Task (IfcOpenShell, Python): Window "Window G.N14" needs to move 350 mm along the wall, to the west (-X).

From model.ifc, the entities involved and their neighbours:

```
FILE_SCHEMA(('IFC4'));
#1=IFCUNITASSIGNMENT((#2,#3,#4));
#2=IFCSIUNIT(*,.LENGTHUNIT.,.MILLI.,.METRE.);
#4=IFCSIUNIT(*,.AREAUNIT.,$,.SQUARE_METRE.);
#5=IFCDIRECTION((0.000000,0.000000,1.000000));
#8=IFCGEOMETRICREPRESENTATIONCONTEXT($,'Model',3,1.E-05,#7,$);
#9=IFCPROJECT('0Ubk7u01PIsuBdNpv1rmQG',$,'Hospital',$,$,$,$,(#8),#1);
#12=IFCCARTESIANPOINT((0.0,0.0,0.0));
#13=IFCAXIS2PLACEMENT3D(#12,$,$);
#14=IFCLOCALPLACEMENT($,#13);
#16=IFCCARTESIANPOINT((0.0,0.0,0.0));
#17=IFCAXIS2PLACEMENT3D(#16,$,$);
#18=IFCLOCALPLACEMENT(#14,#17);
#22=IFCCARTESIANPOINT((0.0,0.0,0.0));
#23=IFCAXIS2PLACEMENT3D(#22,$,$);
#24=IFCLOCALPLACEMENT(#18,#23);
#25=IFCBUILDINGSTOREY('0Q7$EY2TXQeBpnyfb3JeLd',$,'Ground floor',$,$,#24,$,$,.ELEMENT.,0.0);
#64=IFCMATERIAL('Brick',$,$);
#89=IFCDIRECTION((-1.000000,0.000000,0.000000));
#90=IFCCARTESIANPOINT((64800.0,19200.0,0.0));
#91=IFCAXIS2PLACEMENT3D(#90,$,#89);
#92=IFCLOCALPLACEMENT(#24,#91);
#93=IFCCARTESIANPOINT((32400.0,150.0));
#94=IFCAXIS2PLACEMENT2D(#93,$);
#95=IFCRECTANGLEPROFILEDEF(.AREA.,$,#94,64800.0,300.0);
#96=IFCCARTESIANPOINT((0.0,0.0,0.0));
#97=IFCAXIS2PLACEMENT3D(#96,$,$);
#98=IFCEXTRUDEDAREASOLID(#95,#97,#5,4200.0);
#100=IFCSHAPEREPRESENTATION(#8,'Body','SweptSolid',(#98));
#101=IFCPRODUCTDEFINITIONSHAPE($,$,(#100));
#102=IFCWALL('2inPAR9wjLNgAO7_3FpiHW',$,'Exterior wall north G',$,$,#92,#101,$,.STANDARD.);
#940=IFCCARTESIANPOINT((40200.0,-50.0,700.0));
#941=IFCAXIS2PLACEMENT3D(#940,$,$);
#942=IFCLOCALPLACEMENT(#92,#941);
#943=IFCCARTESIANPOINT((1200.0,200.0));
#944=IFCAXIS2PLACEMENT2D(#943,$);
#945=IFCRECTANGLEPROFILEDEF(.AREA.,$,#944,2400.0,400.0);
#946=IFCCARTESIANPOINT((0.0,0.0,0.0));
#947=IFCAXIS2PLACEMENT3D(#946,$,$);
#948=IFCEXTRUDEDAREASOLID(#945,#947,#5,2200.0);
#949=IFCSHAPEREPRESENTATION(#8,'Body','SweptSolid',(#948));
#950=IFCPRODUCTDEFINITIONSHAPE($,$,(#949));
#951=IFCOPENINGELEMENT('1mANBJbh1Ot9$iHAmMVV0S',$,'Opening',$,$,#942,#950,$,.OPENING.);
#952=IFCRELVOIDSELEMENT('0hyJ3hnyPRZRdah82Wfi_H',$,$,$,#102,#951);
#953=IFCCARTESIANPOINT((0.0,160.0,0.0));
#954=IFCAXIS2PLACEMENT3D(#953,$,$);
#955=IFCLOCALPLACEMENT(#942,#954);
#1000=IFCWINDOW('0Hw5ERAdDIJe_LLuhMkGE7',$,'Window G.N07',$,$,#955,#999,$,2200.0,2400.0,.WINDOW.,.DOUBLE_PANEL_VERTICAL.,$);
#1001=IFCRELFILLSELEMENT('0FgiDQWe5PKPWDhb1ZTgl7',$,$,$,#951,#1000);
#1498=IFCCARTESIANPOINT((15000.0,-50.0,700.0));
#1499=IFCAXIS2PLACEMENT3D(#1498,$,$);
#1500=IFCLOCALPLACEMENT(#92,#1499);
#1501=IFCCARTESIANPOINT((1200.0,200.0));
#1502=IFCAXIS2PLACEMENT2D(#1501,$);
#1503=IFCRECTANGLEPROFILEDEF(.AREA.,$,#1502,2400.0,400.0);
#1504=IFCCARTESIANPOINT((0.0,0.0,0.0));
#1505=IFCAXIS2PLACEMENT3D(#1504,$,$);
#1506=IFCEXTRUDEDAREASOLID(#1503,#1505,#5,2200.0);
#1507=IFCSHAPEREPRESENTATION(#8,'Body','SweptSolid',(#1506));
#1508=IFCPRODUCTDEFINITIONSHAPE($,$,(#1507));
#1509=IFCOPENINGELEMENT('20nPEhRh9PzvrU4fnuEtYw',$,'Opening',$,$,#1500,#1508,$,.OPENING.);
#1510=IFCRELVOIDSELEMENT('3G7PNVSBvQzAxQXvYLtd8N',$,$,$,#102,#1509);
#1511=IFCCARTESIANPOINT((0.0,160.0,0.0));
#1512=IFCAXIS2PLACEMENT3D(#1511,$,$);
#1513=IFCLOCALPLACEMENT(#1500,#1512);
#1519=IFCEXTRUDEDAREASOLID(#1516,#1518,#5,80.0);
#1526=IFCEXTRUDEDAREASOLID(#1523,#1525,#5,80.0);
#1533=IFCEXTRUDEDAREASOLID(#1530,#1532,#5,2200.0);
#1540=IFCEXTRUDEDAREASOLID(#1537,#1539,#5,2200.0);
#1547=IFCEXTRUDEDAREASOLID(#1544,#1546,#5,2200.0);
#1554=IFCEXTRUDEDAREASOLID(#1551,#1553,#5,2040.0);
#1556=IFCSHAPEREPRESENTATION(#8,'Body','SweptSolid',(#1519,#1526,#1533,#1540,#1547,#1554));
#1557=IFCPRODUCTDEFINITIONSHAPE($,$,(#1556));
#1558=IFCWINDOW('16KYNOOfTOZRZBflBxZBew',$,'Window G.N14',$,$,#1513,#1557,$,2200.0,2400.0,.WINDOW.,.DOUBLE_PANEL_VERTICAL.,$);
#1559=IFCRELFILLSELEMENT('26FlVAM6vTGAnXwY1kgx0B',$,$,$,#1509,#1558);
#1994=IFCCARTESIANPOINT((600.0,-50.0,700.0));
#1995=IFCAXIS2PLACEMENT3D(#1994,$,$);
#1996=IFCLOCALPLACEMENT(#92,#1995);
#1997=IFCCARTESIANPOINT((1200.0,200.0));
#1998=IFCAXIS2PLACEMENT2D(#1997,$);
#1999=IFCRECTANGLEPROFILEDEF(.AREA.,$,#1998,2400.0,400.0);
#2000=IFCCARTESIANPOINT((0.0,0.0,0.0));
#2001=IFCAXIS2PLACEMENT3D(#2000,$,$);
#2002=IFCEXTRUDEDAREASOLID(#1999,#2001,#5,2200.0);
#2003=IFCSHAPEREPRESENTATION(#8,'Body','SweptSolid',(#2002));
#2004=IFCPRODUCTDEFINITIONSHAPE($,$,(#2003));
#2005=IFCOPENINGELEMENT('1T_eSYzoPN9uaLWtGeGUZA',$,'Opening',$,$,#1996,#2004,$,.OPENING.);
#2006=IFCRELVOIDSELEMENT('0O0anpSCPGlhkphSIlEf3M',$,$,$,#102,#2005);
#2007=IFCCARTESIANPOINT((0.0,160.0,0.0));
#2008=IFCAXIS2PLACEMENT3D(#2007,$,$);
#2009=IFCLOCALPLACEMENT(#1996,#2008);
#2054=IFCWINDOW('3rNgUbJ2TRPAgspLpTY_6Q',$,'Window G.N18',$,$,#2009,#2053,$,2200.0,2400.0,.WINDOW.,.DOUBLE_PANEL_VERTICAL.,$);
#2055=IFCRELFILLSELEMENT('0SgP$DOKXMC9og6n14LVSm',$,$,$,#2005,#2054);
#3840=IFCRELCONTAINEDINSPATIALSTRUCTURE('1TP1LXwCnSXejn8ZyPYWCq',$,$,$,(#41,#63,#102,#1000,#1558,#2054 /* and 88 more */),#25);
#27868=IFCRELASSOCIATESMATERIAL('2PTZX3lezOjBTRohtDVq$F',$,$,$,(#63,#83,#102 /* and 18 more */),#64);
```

```python
import ifcopenshell
import ifcopenshell.api.geometry
import ifcopenshell.util.placement
import ifcopenshell.util.unit

model = ifcopenshell.open("model.ifc")
unit_scale = ifcopenshell.util.unit.calculate_unit_scale(model)

window = model.by_guid("16KYNOOfTOZRZBflBxZBew")
opening = window.FillsVoids[0].RelatingOpeningElement
wall = opening.VoidsElements[0].RelatingBuildingElement

wall_matrix = ifcopenshell.util.placement.get_local_placement(wall.ObjectPlacement)
shift = wall_matrix[:3, 0] * 0.35 / unit_scale
before = ifcopenshell.util.placement.get_local_placement(window.ObjectPlacement)[:3, 3].copy()

# The window is placed relative to its opening, so it follows when the opening moves.
matrix = ifcopenshell.util.placement.get_local_placement(opening.ObjectPlacement)
matrix[:3, 3] += shift
ifcopenshell.api.geometry.edit_object_placement(
    model, product=opening, matrix=matrix, is_si=False, should_transform_children=True
)

after = ifcopenshell.util.placement.get_local_placement(window.ObjectPlacement)[:3, 3]
print("window moved by", (after - before).round(3) + 0.0)

model.write("model_v2.ifc")
```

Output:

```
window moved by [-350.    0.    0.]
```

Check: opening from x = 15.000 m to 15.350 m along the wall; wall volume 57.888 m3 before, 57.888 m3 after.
